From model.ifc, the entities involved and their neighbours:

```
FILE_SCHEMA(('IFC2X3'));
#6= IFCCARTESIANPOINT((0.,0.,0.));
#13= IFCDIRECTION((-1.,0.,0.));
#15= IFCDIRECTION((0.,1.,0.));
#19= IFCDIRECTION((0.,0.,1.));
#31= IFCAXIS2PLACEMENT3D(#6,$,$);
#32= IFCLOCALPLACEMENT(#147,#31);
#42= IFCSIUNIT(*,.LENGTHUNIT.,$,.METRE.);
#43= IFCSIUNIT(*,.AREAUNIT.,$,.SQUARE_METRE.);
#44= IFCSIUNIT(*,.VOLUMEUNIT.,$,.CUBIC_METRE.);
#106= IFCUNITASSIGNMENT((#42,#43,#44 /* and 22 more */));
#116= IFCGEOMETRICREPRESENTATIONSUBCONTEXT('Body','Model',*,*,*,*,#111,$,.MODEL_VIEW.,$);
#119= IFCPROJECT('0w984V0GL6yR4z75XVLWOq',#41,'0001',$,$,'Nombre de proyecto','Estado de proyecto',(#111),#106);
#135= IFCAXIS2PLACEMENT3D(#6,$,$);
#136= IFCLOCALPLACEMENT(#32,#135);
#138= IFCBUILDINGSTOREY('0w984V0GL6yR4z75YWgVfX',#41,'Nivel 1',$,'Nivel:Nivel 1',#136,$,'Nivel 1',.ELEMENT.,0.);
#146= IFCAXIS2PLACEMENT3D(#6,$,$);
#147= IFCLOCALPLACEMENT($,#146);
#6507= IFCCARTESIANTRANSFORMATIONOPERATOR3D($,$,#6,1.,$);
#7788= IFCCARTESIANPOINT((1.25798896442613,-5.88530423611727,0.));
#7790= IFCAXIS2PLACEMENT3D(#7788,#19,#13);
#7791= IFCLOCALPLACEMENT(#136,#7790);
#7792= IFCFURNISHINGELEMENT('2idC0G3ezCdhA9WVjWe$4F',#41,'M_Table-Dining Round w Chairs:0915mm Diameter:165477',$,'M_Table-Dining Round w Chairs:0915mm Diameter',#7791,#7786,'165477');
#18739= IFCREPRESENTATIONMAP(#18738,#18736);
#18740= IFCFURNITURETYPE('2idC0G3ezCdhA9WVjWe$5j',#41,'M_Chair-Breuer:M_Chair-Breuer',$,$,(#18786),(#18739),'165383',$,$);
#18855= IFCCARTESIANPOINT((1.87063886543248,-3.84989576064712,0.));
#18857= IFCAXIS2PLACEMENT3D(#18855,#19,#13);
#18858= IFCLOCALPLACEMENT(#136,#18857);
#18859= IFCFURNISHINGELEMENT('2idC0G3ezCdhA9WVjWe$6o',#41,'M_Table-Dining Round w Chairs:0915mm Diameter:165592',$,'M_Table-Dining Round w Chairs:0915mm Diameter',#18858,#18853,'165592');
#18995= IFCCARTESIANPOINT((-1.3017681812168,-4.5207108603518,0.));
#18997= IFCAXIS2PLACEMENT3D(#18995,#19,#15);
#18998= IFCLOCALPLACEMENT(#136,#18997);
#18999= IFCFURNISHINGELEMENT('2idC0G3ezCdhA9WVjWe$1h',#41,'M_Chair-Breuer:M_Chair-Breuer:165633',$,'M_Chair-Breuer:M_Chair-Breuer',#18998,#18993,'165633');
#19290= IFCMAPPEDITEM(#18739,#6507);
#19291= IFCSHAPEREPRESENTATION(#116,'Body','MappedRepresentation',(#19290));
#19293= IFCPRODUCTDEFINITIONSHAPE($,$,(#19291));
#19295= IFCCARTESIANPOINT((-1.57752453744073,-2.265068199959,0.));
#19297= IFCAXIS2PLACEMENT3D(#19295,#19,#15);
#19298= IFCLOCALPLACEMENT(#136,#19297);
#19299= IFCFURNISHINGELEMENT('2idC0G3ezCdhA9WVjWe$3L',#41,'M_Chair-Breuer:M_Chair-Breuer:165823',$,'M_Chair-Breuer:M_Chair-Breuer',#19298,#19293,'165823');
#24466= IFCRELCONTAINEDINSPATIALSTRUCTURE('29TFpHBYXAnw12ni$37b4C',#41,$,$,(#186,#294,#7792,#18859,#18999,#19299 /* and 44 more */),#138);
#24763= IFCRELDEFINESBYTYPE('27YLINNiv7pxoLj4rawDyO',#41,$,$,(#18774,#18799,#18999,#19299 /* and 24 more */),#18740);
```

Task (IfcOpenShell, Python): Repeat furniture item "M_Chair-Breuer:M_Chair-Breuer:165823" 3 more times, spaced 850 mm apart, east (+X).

```python
import numpy as np
import ifcopenshell
import ifcopenshell.api.geometry
import ifcopenshell.api.root
import ifcopenshell.util.element
import ifcopenshell.util.placement

model = ifcopenshell.open("model.ifc")


def reuse_history(source, copy):
    """copy_class also copies each property set's owner history, people and application; keep the originals."""
    for rel in copy.IsDefinedBy:
        if rel.is_a("IfcRelDefinesByProperties") and (history := rel.RelatingPropertyDefinition.OwnerHistory):
            rel.RelatingPropertyDefinition.OwnerHistory = source.OwnerHistory
            ifcopenshell.util.element.remove_deep2(model, history)


source = model.by_id(19299)
base = ifcopenshell.util.placement.get_local_placement(source.ObjectPlacement)
step = np.array([1.0, 0.0, 0.0]) * 0.85

for i in range(1, 4):
    copy = ifcopenshell.api.root.copy_class(model, product=source)
    copy.Representation = ifcopenshell.util.element.copy_deep(
        model, source.Representation, exclude=["IfcGeometricRepresentationContext", "IfcRepresentationMap"]
    )
    copy.Name = "M_Chair-Breuer:M_Chair-Breuer"
    copy.Tag = None
    reuse_history(source, copy)
    matrix = base.copy()
    matrix[:3, 3] += i * step
    print("added at", matrix[:3, 3].round(3) + 0.0)
    ifcopenshell.api.geometry.edit_object_placement(model, product=copy, matrix=matrix, is_si=False)

model.write("model_updated.ifc")
```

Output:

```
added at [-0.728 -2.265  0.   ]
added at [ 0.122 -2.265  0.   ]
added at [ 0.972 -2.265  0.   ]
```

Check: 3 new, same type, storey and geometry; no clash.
